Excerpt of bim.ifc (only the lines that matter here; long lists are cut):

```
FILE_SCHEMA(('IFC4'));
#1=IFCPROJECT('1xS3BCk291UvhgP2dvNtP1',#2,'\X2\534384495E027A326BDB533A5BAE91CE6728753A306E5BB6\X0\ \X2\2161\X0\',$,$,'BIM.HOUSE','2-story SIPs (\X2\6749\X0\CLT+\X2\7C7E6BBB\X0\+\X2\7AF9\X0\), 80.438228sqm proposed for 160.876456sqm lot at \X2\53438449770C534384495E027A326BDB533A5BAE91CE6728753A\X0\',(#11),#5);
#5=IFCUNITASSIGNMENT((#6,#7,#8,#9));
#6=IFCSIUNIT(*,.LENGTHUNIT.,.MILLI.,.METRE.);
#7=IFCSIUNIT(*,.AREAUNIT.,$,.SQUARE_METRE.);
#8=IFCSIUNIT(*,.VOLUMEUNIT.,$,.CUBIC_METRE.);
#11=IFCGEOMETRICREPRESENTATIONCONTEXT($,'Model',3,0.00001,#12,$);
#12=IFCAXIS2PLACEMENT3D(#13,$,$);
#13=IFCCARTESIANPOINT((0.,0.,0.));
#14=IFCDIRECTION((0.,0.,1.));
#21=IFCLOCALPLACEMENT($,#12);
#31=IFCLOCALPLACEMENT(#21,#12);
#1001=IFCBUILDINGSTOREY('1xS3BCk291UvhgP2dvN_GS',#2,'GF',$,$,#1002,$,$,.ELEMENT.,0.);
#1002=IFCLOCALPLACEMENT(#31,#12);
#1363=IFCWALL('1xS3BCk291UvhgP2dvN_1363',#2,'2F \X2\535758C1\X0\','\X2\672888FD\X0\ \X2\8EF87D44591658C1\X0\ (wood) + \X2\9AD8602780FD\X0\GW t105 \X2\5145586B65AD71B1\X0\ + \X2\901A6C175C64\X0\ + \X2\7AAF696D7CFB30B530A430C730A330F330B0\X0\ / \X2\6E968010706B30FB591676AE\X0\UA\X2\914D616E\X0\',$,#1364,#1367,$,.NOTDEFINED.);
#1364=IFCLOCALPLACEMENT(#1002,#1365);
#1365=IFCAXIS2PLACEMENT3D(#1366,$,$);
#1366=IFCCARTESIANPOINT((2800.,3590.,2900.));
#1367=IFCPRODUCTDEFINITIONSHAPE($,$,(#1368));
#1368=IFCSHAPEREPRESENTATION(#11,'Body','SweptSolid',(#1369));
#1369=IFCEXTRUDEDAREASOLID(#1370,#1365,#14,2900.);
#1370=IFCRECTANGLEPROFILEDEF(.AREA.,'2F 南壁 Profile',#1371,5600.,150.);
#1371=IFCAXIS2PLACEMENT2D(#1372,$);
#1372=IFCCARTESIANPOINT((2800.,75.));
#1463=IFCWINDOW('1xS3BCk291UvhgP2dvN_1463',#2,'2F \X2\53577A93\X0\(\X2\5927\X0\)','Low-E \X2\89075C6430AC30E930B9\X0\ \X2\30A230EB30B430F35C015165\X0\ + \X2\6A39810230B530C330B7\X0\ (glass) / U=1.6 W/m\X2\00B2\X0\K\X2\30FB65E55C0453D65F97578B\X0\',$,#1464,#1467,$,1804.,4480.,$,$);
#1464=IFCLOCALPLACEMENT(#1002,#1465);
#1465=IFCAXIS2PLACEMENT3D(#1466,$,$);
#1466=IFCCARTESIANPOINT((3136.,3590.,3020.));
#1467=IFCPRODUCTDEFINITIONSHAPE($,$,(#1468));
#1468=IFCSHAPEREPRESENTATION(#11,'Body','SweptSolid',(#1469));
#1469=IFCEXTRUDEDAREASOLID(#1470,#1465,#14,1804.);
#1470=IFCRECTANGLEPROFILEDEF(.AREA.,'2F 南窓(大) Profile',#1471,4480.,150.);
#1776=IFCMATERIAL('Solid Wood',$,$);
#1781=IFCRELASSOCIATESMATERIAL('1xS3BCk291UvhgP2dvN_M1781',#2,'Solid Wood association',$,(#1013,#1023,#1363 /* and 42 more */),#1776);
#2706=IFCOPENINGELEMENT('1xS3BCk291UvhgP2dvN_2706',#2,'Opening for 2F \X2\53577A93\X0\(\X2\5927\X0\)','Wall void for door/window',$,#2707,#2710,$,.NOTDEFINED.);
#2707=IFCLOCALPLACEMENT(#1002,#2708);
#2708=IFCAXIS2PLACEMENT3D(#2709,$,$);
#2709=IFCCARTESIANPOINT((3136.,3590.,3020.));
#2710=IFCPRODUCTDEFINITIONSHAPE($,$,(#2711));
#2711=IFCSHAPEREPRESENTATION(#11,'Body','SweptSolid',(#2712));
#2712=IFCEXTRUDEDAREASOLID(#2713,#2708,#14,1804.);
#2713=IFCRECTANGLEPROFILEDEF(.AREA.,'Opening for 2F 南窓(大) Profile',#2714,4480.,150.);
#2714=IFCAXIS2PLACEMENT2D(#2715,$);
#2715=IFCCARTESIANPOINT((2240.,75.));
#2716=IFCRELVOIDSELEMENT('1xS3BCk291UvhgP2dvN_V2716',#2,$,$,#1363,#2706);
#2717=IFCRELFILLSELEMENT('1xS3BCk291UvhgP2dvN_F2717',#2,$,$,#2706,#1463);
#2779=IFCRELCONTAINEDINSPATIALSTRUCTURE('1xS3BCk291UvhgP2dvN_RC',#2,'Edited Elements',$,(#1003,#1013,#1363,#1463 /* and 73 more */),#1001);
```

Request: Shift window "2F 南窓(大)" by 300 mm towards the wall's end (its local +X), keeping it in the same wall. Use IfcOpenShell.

```python
import ifcopenshell
import ifcopenshell.api.geometry
import ifcopenshell.util.placement
import ifcopenshell.util.unit

model = ifcopenshell.open("bim.ifc")
unit_scale = ifcopenshell.util.unit.calculate_unit_scale(model)

window = model.by_guid("1xS3BCk291UvhgP2dvN_1463")
opening = window.FillsVoids[0].RelatingOpeningElement
wall = opening.VoidsElements[0].RelatingBuildingElement

wall_matrix = ifcopenshell.util.placement.get_local_placement(wall.ObjectPlacement)
shift = wall_matrix[:3, 0] * 0.3 / unit_scale
before = ifcopenshell.util.placement.get_local_placement(window.ObjectPlacement)[:3, 3].copy()

# The window is not placed relative to its opening, so move both.
for product in (opening, window):
    matrix = ifcopenshell.util.placement.get_local_placement(product.ObjectPlacement)
    matrix[:3, 3] += shift
    ifcopenshell.api.geometry.edit_object_placement(model, product=product, matrix=matrix, is_si=False)

after = ifcopenshell.util.placement.get_local_placement(window.ObjectPlacement)[:3, 3]
print("window moved by", (after - before).round(3) + 0.0)

model.write("bim_rev.ifc")
```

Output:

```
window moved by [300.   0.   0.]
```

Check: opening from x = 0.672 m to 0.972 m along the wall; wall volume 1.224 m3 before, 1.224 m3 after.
